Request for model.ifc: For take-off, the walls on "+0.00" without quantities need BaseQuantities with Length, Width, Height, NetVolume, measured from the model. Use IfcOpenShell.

First a look at what the model holds.

```python
import ifcopenshell
import ifcopenshell.util.element
import ifcopenshell.util.unit

model = ifcopenshell.open("model.ifc")
print(model.schema)
for unit_type in ("LENGTHUNIT", "AREAUNIT", "VOLUMEUNIT"):
    print(unit_type, ifcopenshell.util.unit.calculate_unit_scale(model, unit_type))
storey = next(s for s in model.by_type("IfcBuildingStorey") if s.Name == "+0.00")
walls = [e for e in ifcopenshell.util.element.get_decomposition(storey) if e.is_a("IfcWall")]
for e in sorted(walls, key=lambda e: e.id()):
    print(e.id(), e.is_a(), e.Name, list(ifcopenshell.util.element.get_psets(e, qtos_only=True)), sep=" | ")
```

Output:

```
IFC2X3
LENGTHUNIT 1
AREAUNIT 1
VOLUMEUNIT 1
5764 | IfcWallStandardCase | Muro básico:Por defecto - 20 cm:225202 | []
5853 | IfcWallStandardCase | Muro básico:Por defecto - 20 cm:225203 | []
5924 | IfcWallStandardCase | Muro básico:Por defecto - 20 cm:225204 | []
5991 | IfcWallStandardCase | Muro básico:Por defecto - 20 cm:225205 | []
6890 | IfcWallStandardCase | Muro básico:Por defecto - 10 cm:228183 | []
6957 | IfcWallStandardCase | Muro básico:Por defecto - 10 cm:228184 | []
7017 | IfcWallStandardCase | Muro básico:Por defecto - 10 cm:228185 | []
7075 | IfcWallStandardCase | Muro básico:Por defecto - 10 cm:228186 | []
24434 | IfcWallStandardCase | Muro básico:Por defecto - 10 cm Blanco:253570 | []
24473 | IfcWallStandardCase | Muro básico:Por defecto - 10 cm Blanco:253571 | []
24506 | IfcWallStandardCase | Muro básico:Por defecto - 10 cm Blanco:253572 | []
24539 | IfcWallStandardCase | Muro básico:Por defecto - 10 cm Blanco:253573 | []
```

```python
import ifcopenshell
import ifcopenshell.api.pset
import ifcopenshell.geom
import ifcopenshell.util.element
import ifcopenshell.util.shape
import ifcopenshell.util.unit

model = ifcopenshell.open("model.ifc")
unit_scale = ifcopenshell.util.unit.calculate_unit_scale(model)
volume_scale = ifcopenshell.util.unit.calculate_unit_scale(model, "VOLUMEUNIT")
settings = ifcopenshell.geom.settings()

storey = next(s for s in model.by_type("IfcBuildingStorey") if s.Name == "+0.00")
walls = [e for e in ifcopenshell.util.element.get_decomposition(storey) if e.is_a("IfcWall")]

for e in sorted(walls, key=lambda e: e.id()):
    if ifcopenshell.util.element.get_psets(e, qtos_only=True, should_inherit=False):
        continue
    # Geometry comes back in metres, in the element's own axes.
    shape = ifcopenshell.geom.create_shape(settings, e)
    values = {
        "Length": ifcopenshell.util.shape.get_x(shape.geometry) / unit_scale,
        "Width": ifcopenshell.util.shape.get_y(shape.geometry) / unit_scale,
        "Height": ifcopenshell.util.shape.get_z(shape.geometry) / unit_scale,
        "NetVolume": ifcopenshell.util.shape.get_volume(shape.geometry) / volume_scale,
    }
    qto = ifcopenshell.api.pset.add_qto(model, product=e, name="BaseQuantities")
    ifcopenshell.api.pset.edit_qto(model, qto=qto, properties=values)
    print(e.id(), {k: round(v, 3) for k, v in values.items()})

model.write("model_edited.ifc")
```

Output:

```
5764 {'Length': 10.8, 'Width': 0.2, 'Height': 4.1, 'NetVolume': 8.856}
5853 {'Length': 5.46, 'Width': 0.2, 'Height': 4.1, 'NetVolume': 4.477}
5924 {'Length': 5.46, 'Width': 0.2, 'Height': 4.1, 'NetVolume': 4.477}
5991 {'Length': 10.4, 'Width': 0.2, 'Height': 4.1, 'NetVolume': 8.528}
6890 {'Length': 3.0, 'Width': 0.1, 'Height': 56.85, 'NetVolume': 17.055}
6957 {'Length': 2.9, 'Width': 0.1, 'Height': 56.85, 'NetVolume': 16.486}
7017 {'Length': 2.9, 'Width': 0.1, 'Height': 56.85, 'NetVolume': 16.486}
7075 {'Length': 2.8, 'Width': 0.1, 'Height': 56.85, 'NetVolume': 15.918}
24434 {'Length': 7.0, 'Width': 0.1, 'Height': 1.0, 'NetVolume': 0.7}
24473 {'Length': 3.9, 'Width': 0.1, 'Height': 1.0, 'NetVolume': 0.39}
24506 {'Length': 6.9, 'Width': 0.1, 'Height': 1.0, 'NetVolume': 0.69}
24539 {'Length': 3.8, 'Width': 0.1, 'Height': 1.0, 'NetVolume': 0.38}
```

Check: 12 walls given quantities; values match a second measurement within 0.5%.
